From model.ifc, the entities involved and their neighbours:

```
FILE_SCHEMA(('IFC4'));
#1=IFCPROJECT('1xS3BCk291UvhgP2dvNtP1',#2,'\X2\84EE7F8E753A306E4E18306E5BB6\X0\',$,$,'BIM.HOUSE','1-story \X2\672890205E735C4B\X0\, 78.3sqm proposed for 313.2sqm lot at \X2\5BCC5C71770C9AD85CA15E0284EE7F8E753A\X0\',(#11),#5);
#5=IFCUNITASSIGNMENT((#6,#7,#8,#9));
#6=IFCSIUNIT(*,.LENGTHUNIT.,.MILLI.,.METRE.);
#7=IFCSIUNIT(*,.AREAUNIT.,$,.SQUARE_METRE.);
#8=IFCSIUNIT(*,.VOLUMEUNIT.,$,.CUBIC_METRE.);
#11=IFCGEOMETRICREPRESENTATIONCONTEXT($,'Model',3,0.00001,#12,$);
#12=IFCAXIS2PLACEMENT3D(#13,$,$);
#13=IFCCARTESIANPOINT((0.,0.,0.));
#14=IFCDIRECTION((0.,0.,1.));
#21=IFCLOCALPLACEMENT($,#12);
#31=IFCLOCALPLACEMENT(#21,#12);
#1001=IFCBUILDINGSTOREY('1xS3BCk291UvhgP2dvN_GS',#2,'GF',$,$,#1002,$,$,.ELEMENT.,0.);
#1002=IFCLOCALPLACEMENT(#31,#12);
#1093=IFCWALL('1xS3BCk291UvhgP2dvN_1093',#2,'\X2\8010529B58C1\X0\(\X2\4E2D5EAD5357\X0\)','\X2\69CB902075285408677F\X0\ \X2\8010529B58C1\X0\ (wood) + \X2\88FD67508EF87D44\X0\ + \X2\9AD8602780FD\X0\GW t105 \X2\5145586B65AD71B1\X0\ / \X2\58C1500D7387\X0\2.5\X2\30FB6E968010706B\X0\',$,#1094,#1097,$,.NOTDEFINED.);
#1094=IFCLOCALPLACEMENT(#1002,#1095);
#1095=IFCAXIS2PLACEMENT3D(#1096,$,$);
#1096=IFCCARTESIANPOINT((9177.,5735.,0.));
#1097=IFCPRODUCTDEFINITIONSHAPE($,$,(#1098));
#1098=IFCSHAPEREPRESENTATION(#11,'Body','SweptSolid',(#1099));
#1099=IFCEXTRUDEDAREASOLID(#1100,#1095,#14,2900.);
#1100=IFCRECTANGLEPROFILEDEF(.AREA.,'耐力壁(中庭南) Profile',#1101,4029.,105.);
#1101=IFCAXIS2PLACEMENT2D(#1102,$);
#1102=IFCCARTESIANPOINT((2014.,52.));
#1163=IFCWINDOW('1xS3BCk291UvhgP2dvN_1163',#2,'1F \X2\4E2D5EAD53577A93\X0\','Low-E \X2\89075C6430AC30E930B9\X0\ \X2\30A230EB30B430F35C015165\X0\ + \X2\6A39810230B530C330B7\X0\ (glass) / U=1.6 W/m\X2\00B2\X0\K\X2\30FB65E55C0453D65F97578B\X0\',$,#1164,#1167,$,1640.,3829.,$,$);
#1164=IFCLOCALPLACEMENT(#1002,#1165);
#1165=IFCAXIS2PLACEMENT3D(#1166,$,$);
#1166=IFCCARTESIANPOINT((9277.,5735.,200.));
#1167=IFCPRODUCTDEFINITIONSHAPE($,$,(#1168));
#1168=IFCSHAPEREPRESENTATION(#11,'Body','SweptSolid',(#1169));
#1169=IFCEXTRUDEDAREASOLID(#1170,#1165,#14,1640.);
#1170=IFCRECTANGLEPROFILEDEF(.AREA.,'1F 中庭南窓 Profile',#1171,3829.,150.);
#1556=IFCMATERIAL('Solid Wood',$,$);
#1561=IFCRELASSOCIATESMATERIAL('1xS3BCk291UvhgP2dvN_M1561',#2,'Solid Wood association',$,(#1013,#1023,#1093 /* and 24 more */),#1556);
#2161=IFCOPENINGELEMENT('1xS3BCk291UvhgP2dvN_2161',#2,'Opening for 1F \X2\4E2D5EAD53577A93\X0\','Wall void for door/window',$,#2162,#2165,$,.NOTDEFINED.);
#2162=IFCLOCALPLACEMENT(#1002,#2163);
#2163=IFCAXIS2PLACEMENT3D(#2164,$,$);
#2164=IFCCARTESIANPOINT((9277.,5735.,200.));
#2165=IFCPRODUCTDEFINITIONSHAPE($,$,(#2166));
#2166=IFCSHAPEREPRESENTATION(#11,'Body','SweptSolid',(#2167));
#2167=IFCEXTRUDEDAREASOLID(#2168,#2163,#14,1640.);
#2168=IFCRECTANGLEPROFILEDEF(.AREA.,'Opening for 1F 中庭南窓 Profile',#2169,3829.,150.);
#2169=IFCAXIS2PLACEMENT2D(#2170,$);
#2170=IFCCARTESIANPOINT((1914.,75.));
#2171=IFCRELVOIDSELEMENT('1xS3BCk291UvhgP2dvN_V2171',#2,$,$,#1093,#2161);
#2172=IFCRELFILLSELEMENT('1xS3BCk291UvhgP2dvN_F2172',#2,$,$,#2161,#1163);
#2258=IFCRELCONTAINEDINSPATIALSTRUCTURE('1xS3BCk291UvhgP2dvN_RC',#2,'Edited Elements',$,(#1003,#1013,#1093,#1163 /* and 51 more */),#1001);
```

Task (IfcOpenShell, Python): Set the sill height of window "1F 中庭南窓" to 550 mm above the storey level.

```python
import numpy as np
import ifcopenshell
import ifcopenshell.api.geometry
import ifcopenshell.geom
import ifcopenshell.util.element
import ifcopenshell.util.placement
import ifcopenshell.util.shape
import ifcopenshell.util.unit

model = ifcopenshell.open("model.ifc")
unit_scale = ifcopenshell.util.unit.calculate_unit_scale(model)

window = model.by_id(1163)
opening = window.FillsVoids[0].RelatingOpeningElement
storey = ifcopenshell.util.element.get_container(window, ifc_class="IfcBuildingStorey")
level = ifcopenshell.util.placement.get_local_placement(storey.ObjectPlacement)[2, 3]

# The opening's origin need not be at the sill, so measure its lowest point.
shape = ifcopenshell.geom.create_shape(ifcopenshell.geom.settings(), opening)
bottom = ifcopenshell.util.shape.get_shape_bottom_elevation(shape, shape.geometry) / unit_scale
dz = level + 0.55 / unit_scale - bottom

shift = np.array([0.0, 0.0, dz])
# The window is not placed relative to its opening, so move both.
for product in (opening, window):
    matrix = ifcopenshell.util.placement.get_local_placement(product.ObjectPlacement)
    matrix[:3, 3] += shift
    ifcopenshell.api.geometry.edit_object_placement(model, product=product, matrix=matrix, is_si=False)

print(f"moved by {dz * unit_scale:+.3f} m")

model.write("model_updated.ifc")
```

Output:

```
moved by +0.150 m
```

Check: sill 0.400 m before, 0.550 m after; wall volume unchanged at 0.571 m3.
